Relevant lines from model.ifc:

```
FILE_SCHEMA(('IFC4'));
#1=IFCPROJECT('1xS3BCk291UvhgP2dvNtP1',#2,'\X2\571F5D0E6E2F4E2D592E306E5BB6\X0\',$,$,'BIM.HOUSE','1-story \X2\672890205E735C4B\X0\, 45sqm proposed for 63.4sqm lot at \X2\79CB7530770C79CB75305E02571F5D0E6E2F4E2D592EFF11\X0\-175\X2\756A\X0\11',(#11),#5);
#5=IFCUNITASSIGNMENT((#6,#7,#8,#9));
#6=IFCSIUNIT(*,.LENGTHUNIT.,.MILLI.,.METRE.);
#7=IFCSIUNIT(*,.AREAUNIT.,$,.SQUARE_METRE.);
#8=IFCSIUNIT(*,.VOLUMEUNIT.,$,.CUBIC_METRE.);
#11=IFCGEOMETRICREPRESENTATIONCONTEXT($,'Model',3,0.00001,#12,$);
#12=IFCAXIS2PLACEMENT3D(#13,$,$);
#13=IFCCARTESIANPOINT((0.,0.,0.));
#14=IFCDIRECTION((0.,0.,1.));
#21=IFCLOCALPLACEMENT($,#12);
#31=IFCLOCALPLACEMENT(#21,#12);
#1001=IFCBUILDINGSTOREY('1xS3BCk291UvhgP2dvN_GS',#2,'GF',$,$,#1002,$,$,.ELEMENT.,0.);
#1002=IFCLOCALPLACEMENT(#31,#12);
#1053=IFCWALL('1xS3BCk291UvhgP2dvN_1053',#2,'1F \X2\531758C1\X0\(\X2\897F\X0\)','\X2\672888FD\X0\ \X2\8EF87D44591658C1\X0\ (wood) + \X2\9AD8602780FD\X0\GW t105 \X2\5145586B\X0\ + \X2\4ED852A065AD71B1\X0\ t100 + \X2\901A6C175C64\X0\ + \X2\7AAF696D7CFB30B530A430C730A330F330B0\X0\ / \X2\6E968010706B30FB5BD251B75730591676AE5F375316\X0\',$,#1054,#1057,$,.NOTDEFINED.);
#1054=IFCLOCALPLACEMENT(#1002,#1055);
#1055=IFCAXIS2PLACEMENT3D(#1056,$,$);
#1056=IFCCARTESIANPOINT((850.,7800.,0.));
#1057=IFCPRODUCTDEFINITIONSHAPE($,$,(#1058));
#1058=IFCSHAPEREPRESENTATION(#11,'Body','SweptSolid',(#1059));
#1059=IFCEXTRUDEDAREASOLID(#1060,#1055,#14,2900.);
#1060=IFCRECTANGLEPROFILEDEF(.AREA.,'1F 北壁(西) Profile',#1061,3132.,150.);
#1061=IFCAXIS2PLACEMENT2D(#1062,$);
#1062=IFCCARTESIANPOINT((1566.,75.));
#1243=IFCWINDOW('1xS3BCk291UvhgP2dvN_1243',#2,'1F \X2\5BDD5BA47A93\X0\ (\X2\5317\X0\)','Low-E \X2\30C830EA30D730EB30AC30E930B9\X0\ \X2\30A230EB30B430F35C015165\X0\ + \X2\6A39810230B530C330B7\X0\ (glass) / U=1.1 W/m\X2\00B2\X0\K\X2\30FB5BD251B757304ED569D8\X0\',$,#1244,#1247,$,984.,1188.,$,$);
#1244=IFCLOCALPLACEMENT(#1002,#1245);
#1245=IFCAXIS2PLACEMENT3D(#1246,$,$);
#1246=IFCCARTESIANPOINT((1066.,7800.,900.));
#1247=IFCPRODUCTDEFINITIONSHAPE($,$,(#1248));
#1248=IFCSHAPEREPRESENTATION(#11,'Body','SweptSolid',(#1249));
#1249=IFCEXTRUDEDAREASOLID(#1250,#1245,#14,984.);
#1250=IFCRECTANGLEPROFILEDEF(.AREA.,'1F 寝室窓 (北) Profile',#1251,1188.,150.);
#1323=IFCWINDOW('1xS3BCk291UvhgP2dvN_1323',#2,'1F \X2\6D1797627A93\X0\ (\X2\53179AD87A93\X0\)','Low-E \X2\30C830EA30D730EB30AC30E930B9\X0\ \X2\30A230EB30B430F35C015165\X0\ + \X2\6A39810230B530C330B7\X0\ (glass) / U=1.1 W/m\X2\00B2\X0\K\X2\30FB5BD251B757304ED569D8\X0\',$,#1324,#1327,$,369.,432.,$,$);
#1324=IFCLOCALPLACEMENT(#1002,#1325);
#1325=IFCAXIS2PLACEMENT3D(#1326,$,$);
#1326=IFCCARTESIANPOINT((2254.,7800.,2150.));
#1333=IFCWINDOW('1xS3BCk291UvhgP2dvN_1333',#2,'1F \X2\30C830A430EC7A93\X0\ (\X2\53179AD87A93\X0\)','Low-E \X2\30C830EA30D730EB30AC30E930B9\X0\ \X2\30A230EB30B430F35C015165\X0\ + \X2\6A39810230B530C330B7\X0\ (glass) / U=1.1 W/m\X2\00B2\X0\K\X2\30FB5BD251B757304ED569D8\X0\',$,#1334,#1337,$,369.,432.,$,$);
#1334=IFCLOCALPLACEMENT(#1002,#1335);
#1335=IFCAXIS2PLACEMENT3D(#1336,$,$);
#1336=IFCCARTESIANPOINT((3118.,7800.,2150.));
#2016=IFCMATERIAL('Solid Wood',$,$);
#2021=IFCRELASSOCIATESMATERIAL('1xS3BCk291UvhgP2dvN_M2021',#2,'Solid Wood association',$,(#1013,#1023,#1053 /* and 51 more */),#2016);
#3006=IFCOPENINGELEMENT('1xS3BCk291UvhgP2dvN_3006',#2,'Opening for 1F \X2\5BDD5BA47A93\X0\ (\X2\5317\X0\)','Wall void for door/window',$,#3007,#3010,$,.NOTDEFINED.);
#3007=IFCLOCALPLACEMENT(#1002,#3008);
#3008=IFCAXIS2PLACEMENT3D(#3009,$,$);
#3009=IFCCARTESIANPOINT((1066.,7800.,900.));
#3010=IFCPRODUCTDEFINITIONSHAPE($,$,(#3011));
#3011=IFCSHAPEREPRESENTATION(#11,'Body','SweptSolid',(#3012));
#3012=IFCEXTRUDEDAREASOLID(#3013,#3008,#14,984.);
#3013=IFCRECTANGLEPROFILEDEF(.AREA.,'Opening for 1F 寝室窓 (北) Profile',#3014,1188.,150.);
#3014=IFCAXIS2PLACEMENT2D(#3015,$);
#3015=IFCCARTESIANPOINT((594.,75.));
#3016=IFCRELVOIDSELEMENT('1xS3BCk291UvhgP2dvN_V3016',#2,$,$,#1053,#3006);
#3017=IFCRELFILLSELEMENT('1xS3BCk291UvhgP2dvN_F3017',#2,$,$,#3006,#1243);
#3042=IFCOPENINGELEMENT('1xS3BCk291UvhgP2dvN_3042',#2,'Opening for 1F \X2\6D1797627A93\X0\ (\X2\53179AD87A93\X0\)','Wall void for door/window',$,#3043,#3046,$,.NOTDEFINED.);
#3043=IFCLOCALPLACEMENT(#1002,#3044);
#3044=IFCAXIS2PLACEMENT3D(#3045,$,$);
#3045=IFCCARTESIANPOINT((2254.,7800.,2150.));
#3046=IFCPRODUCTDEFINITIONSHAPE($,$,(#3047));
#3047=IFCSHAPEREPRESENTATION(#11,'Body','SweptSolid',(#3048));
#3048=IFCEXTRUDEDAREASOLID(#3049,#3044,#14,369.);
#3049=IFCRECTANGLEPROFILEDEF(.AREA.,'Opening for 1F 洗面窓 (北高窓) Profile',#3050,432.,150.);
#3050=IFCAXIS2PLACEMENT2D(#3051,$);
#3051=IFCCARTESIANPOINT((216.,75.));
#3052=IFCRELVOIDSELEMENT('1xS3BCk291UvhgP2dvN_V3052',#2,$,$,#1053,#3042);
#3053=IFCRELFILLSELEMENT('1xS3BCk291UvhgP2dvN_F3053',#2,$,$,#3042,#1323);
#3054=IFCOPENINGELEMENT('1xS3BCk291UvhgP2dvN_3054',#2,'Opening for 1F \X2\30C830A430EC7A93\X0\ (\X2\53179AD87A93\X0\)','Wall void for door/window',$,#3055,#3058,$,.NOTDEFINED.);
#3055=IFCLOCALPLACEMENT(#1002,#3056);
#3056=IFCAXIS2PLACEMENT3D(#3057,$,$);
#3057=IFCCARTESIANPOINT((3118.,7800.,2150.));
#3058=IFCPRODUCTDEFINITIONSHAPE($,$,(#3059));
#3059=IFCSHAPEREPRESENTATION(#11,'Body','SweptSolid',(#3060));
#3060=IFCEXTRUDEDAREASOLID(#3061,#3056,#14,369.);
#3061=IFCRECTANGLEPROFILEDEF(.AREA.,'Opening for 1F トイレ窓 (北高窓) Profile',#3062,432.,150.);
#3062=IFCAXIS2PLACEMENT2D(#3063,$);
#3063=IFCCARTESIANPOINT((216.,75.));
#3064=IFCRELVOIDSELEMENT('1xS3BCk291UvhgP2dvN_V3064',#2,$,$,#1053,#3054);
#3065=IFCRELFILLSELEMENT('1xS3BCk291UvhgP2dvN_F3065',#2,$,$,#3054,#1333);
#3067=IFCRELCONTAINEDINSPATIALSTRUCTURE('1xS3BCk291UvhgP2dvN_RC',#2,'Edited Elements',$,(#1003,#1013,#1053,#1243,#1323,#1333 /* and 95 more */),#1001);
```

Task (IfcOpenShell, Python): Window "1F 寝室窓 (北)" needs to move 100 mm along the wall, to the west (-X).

```python
import ifcopenshell
import ifcopenshell.api.geometry
import ifcopenshell.util.placement

model = ifcopenshell.open("model.ifc")

window = model.by_guid("1xS3BCk291UvhgP2dvN_1243")
opening = window.FillsVoids[0].RelatingOpeningElement
wall = opening.VoidsElements[0].RelatingBuildingElement

wall_matrix = ifcopenshell.util.placement.get_local_placement(wall.ObjectPlacement)
shift = wall_matrix[:3, 0] * -100.0
before = ifcopenshell.util.placement.get_local_placement(window.ObjectPlacement)[:3, 3].copy()

# The window is not placed relative to its opening, so move both.
for product in (opening, window):
    matrix = ifcopenshell.util.placement.get_local_placement(product.ObjectPlacement)
    matrix[:3, 3] += shift
    ifcopenshell.api.geometry.edit_object_placement(model, product=product, matrix=matrix, is_si=False)

after = ifcopenshell.util.placement.get_local_placement(window.ObjectPlacement)[:3, 3]
print("window moved by", (after - before).round(3) + 0.0)

model.write("model_edited.ifc")
```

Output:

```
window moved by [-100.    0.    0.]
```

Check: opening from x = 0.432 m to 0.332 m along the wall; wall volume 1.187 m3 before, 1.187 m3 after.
